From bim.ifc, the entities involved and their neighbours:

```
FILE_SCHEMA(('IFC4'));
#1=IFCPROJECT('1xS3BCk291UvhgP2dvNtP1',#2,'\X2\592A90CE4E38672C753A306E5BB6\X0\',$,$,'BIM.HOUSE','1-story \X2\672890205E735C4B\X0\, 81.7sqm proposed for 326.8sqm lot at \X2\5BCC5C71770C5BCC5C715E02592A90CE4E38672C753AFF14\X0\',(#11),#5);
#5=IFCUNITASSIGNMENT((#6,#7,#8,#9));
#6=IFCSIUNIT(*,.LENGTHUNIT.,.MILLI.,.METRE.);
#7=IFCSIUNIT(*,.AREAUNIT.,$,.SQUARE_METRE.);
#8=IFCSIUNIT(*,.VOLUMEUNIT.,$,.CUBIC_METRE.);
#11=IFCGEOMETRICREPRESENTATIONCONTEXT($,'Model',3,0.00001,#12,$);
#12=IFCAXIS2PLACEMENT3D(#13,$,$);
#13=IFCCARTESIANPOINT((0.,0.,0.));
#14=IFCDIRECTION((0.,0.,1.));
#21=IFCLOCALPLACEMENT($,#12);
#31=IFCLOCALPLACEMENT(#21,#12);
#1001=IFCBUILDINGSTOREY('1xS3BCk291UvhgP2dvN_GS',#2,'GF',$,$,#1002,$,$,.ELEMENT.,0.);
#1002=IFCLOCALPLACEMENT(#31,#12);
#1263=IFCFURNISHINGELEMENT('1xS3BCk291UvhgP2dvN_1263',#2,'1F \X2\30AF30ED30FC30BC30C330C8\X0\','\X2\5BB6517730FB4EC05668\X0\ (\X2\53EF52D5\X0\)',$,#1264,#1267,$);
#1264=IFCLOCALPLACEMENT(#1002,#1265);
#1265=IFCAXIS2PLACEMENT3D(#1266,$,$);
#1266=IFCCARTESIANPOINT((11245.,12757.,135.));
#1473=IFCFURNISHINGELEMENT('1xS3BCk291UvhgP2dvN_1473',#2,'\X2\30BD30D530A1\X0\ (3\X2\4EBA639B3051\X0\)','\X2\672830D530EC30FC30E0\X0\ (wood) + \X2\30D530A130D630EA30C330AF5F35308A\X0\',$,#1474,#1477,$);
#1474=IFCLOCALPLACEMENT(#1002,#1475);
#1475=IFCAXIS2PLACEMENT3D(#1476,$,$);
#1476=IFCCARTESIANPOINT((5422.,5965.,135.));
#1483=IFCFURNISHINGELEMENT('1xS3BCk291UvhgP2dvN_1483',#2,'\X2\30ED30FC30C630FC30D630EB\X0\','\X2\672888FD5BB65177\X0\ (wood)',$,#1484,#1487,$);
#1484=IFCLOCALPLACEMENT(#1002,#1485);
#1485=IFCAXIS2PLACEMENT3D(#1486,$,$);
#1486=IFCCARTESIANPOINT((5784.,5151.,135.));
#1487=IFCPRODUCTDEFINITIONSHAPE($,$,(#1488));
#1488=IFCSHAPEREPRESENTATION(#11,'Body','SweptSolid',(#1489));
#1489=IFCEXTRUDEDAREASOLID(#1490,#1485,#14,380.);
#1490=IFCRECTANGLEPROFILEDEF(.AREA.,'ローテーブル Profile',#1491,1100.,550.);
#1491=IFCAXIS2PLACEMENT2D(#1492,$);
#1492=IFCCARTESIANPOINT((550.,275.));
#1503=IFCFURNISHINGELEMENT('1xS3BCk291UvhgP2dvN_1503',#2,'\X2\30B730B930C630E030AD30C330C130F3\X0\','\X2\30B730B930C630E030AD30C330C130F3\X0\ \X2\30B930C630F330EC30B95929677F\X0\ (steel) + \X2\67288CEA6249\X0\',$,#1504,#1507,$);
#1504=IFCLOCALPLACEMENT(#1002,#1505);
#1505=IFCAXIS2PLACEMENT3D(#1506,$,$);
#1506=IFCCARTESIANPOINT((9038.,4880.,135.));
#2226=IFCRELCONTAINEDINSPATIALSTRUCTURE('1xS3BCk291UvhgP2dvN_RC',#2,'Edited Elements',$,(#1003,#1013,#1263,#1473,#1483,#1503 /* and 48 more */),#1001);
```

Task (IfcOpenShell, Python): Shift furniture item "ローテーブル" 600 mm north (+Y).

```python
import ifcopenshell
import ifcopenshell.api.geometry
import ifcopenshell.util.placement
import ifcopenshell.util.unit

model = ifcopenshell.open("bim.ifc")
unit_scale = ifcopenshell.util.unit.calculate_unit_scale(model)

item = model.by_id(1483)
matrix = ifcopenshell.util.placement.get_local_placement(item.ObjectPlacement)
matrix[1, 3] += 0.6 / unit_scale
ifcopenshell.api.geometry.edit_object_placement(model, product=item, matrix=matrix, is_si=False)

print(ifcopenshell.util.placement.get_local_placement(item.ObjectPlacement).round(3) + 0.0)

model.write("bim-out.ifc")
```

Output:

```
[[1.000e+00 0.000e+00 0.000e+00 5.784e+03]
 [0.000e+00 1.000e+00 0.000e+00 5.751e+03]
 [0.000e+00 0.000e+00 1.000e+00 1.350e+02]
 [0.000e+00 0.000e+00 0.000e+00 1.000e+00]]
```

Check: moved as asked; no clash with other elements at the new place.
